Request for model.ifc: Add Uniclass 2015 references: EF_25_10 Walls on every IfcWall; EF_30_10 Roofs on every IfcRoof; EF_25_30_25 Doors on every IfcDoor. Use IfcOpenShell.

First a look at what the model holds.

```python
import ifcopenshell

model = ifcopenshell.open("model.ifc")
print(model.schema)
print("classifications:", [c.Name for c in model.by_type("IfcClassification")])
for ifc_class in ("IfcDoor", "IfcRoof", "IfcStair", "IfcWall", "IfcWindow"):
    print(ifc_class, len(model.by_type(ifc_class)))
```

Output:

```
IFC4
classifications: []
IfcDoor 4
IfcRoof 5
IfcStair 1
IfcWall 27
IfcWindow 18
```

```python
import ifcopenshell
import ifcopenshell.api.classification

model = ifcopenshell.open("model.ifc")

system = ifcopenshell.api.classification.add_classification(model, classification="Uniclass 2015")

codes = {
    "IfcWall": ("EF_25_10", "Walls"),
    "IfcRoof": ("EF_30_10", "Roofs"),
    "IfcDoor": ("EF_25_30_25", "Doors"),
}
for ifc_class, (code, name) in codes.items():
    products = model.by_type(ifc_class)
    ifcopenshell.api.classification.add_reference(
        model, products=products, classification=system, identification=code, name=name
    )
    print(code, len(products))

model.write("model_edited.ifc")
```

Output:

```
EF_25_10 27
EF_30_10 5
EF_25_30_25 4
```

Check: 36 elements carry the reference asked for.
